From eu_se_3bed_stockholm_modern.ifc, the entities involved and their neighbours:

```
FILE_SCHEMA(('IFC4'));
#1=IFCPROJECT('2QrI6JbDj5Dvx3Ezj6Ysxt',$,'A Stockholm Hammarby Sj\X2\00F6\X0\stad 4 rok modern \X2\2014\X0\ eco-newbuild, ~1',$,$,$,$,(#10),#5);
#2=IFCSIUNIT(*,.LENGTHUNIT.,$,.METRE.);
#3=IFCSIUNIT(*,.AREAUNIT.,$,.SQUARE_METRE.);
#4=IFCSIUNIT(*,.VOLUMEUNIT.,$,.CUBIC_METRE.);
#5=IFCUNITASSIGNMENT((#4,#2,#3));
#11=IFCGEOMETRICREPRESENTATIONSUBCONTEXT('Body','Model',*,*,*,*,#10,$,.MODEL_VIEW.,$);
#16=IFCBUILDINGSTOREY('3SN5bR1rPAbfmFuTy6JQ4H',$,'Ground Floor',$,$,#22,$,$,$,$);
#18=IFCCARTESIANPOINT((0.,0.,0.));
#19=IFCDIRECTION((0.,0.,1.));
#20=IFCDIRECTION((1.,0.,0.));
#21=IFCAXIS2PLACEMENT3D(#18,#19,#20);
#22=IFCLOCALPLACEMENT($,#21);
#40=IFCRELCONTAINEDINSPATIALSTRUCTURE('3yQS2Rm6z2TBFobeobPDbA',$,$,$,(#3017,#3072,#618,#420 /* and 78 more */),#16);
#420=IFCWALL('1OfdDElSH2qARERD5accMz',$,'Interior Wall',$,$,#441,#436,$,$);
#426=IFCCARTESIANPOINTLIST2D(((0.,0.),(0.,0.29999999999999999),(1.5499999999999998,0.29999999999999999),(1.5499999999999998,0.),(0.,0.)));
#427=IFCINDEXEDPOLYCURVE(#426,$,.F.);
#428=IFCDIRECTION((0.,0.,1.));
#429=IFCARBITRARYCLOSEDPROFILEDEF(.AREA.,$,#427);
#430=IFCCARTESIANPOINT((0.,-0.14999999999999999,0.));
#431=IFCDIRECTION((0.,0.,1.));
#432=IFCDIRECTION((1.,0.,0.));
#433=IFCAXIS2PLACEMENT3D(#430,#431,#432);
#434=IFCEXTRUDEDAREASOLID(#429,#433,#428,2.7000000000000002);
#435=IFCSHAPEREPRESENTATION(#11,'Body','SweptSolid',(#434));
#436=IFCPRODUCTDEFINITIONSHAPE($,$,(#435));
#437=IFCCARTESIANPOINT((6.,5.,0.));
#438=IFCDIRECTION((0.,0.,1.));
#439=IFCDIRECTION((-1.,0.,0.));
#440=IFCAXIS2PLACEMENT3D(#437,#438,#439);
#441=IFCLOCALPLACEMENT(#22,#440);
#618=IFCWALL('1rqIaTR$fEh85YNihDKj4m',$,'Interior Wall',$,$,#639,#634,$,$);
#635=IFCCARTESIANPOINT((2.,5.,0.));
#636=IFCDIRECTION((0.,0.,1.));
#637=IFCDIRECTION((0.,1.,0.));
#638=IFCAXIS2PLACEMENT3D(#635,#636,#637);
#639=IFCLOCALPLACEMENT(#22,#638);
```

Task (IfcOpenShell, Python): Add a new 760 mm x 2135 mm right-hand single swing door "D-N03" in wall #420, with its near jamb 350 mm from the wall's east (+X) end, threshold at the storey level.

```python
import numpy as np
import ifcopenshell
import ifcopenshell.api.feature
import ifcopenshell.api.geometry
import ifcopenshell.api.root
import ifcopenshell.api.spatial
import ifcopenshell.geom
import ifcopenshell.util.element
import ifcopenshell.util.placement
import ifcopenshell.util.representation
import ifcopenshell.util.shape
import ifcopenshell.util.unit

model = ifcopenshell.open("eu_se_3bed_stockholm_modern.ifc")
unit_scale = ifcopenshell.util.unit.calculate_unit_scale(model)
settings = ifcopenshell.geom.settings()


def volume(element):
    """Net volume in cubic metres, openings subtracted."""
    shape = ifcopenshell.geom.create_shape(settings, element)
    return ifcopenshell.util.shape.get_volume(shape.geometry)


wall = model.by_id(420)
storey = ifcopenshell.util.element.get_container(wall, ifc_class="IfcBuildingStorey")
context = ifcopenshell.util.representation.get_context(model, "Model", "Body", "MODEL_VIEW")
before = volume(wall)

width, height, from_end, sill = 0.76, 2.135, 0.35, 0.0  # metres

# The wall runs along its own X axis, and the end named is its -X end.
wall_shape = ifcopenshell.geom.create_shape(settings, wall)
x, y, z = ifcopenshell.util.shape.get_vertices(wall_shape.geometry).T
start = x.min() + from_end
face, thickness = float(y.min()), float(y.max() - y.min())
wall_matrix = ifcopenshell.util.placement.get_local_placement(wall.ObjectPlacement)
level = ifcopenshell.util.placement.get_local_placement(storey.ObjectPlacement)[2, 3]


def in_wall(x, y):
    """Placement at x, y metres in the wall's axes, at sill height."""
    matrix = wall_matrix.copy()
    matrix[:, 3] = wall_matrix @ np.array([x / unit_scale, y / unit_scale, 0.0, 1.0])
    matrix[2, 3] = level + sill / unit_scale
    return matrix


# Opening: a box that overshoots both wall faces by 50 mm.
opening = ifcopenshell.api.root.create_entity(model, ifc_class="IfcOpeningElement", predefined_type="OPENING")
box = ifcopenshell.api.geometry.add_wall_representation(
    model, context=context, length=width, height=height, thickness=thickness + 0.1
)
ifcopenshell.api.geometry.assign_representation(model, product=opening, representation=box)
ifcopenshell.api.geometry.edit_object_placement(model, product=opening, matrix=in_wall(start, face - 0.05), is_si=False)
ifcopenshell.api.feature.add_feature(model, feature=opening, element=wall)

door = ifcopenshell.api.root.create_entity(model, ifc_class="IfcDoor", name="D-N03", predefined_type="DOOR")
door.OverallWidth, door.OverallHeight = width / unit_scale, height / unit_scale
door.OperationType = "SINGLE_SWING_RIGHT"
body = ifcopenshell.api.geometry.add_door_representation(
    model,
    context=context,
    overall_width=door.OverallWidth,
    overall_height=door.OverallHeight,
    operation_type="SINGLE_SWING_RIGHT",
    lining_properties={"LiningDepth": thickness / unit_scale, "ThresholdDepth": thickness / unit_scale},
)
ifcopenshell.api.geometry.assign_representation(model, product=door, representation=body)
ifcopenshell.api.spatial.assign_container(model, products=[door], relating_structure=storey)
ifcopenshell.api.feature.add_filling(model, opening=opening, element=door)

# The lining spans the wall, so the door starts at the wall face.
ifcopenshell.api.geometry.edit_object_placement(model, product=door, matrix=in_wall(start, face), is_si=False)

after = volume(wall)

print(f"wall volume {before:.3f} -> {after:.3f} m3")

model.write("eu_se_3bed_stockholm_modern-out.ifc")
```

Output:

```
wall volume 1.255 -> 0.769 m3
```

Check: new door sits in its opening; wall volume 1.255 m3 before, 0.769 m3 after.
